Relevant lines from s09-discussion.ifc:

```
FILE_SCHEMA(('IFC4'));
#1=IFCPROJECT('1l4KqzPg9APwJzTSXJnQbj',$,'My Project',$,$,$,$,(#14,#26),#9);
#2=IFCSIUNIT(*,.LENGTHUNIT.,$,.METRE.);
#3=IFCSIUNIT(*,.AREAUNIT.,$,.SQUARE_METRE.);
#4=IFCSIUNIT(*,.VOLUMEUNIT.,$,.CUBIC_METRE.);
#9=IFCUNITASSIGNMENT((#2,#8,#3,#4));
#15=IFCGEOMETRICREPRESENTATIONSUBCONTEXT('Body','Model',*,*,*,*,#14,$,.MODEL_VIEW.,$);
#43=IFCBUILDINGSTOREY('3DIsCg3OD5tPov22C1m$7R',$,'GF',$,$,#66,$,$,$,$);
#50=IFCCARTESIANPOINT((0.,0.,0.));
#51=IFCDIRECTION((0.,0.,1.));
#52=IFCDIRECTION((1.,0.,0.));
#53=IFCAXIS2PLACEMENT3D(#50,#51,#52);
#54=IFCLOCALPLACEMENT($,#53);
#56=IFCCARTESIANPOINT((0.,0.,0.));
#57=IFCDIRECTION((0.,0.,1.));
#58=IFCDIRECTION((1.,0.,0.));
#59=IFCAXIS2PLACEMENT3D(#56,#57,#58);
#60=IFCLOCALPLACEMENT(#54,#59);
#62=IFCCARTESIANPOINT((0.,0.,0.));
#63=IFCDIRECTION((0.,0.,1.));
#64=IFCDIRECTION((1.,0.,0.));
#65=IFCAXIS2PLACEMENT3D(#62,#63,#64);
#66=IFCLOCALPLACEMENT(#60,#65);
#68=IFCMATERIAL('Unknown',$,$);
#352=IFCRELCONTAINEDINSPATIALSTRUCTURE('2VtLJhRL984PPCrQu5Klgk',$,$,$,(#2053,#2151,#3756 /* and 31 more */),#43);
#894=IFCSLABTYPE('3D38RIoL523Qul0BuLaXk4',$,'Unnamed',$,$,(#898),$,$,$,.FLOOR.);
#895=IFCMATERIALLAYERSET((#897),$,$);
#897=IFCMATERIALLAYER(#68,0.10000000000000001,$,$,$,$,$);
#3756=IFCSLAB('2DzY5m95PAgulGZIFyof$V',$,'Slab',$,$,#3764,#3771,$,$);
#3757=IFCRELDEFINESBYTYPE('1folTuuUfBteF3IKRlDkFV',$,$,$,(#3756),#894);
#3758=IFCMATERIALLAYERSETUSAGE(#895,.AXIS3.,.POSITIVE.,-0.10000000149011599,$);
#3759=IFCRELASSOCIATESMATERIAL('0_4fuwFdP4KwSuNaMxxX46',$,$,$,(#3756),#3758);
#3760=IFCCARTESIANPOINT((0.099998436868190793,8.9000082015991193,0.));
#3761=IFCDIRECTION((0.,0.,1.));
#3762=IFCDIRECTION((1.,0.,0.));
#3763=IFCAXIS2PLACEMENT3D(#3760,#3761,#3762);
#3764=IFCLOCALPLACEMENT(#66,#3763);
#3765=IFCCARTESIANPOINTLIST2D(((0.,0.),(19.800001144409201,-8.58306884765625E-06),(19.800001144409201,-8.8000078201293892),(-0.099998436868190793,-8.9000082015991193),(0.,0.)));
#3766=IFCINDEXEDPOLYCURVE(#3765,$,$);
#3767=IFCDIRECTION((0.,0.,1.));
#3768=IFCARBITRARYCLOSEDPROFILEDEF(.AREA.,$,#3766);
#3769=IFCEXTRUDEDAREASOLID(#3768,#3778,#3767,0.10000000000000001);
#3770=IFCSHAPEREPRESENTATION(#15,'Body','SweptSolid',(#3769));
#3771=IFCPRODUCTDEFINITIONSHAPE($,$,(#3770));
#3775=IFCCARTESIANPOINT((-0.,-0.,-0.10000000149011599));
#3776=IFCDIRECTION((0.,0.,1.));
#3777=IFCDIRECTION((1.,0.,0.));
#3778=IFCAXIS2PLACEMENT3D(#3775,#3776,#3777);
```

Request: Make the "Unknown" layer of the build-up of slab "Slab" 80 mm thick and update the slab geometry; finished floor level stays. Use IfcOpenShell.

```python
import ifcopenshell
import ifcopenshell.util.element
import ifcopenshell.util.representation

model = ifcopenshell.open("s09-discussion.ifc")

layer_set = model.by_id(895)
layer = next(l for l in layer_set.MaterialLayers if l.Material and l.Material.Name == "Unknown")
change = 0.08 - layer.LayerThickness
layer.LayerThickness += change

# Geometry does not follow the layer set by itself.
slabs = [e for e in ifcopenshell.util.element.get_elements_by_material(model, layer_set) if e.is_a("IfcSlab")]
for slab in sorted(slabs, key=lambda e: e.id()):
    body = ifcopenshell.util.representation.get_representation(slab, "Model", "Body")
    solid = body.Items[0]
    old_depth = solid.Depth
    solid.Depth += change
    # Extruded upwards: lower the start of the extrusion so the top stays.
    x, y, z = solid.Position.Location.Coordinates
    solid.Position.Location = model.createIfcCartesianPoint((x, y, z - change))
    print(slab.id(), f"{old_depth:g} -> {solid.Depth:g}")

# The layers are counted up from the underside, which has moved.
for usage in {ifcopenshell.util.element.get_material(slab) for slab in slabs}:
    usage.OffsetFromReferenceLine -= change

model.write("s09-discussion_v2.ifc")
```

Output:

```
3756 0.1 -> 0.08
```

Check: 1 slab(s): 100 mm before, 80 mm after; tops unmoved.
